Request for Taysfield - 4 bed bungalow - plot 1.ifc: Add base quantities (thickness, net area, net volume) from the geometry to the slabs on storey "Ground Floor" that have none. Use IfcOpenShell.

First a look at what the model holds.

```python
import ifcopenshell
import ifcopenshell.util.element
import ifcopenshell.util.unit

model = ifcopenshell.open("Taysfield - 4 bed bungalow - plot 1.ifc")
print(model.schema)
for unit_type in ("LENGTHUNIT", "AREAUNIT", "VOLUMEUNIT"):
    print(unit_type, ifcopenshell.util.unit.calculate_unit_scale(model, unit_type))
storey = next(s for s in model.by_type("IfcBuildingStorey") if s.Name == "Ground Floor")
slabs = [e for e in ifcopenshell.util.element.get_decomposition(storey) if e.is_a("IfcSlab")]
for e in sorted(slabs, key=lambda e: e.id()):
    print(e.id(), e.is_a(), e.Name, list(ifcopenshell.util.element.get_psets(e, qtos_only=True)), sep=" | ")
```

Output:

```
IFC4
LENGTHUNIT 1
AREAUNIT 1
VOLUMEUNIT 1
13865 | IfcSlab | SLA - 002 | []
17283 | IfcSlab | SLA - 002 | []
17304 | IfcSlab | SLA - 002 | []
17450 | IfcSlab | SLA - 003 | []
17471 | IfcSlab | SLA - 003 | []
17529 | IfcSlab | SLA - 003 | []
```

```python
import ifcopenshell
import ifcopenshell.api.pset
import ifcopenshell.geom
import ifcopenshell.util.element
import ifcopenshell.util.shape
import ifcopenshell.util.unit

model = ifcopenshell.open("Taysfield - 4 bed bungalow - plot 1.ifc")
unit_scale = ifcopenshell.util.unit.calculate_unit_scale(model)
area_scale = ifcopenshell.util.unit.calculate_unit_scale(model, "AREAUNIT")
volume_scale = ifcopenshell.util.unit.calculate_unit_scale(model, "VOLUMEUNIT")
settings = ifcopenshell.geom.settings()

storey = next(s for s in model.by_type("IfcBuildingStorey") if s.Name == "Ground Floor")
slabs = [e for e in ifcopenshell.util.element.get_decomposition(storey) if e.is_a("IfcSlab")]

for e in sorted(slabs, key=lambda e: e.id()):
    if ifcopenshell.util.element.get_psets(e, qtos_only=True, should_inherit=False):
        continue
    # Geometry comes back in metres, in the element's own axes.
    shape = ifcopenshell.geom.create_shape(settings, e)
    values = {
        "Width": ifcopenshell.util.shape.get_z(shape.geometry) / unit_scale,
        "NetArea": ifcopenshell.util.shape.get_footprint_area(shape.geometry) / area_scale,
        "NetVolume": ifcopenshell.util.shape.get_volume(shape.geometry) / volume_scale,
    }
    qto = ifcopenshell.api.pset.add_qto(model, product=e, name="Qto_SlabBaseQuantities")
    ifcopenshell.api.pset.edit_qto(model, qto=qto, properties=values)
    print(e.id(), {k: round(v, 3) for k, v in values.items()})

model.write("Taysfield - 4 bed bungalow - plot 1_v2.ifc")
```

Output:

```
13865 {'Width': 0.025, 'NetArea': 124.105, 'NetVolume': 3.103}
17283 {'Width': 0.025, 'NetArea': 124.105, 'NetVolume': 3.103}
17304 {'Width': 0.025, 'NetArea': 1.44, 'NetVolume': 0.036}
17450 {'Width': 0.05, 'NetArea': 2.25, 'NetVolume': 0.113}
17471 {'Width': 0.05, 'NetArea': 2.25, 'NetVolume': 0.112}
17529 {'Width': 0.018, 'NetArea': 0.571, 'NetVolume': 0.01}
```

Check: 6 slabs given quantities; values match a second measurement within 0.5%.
